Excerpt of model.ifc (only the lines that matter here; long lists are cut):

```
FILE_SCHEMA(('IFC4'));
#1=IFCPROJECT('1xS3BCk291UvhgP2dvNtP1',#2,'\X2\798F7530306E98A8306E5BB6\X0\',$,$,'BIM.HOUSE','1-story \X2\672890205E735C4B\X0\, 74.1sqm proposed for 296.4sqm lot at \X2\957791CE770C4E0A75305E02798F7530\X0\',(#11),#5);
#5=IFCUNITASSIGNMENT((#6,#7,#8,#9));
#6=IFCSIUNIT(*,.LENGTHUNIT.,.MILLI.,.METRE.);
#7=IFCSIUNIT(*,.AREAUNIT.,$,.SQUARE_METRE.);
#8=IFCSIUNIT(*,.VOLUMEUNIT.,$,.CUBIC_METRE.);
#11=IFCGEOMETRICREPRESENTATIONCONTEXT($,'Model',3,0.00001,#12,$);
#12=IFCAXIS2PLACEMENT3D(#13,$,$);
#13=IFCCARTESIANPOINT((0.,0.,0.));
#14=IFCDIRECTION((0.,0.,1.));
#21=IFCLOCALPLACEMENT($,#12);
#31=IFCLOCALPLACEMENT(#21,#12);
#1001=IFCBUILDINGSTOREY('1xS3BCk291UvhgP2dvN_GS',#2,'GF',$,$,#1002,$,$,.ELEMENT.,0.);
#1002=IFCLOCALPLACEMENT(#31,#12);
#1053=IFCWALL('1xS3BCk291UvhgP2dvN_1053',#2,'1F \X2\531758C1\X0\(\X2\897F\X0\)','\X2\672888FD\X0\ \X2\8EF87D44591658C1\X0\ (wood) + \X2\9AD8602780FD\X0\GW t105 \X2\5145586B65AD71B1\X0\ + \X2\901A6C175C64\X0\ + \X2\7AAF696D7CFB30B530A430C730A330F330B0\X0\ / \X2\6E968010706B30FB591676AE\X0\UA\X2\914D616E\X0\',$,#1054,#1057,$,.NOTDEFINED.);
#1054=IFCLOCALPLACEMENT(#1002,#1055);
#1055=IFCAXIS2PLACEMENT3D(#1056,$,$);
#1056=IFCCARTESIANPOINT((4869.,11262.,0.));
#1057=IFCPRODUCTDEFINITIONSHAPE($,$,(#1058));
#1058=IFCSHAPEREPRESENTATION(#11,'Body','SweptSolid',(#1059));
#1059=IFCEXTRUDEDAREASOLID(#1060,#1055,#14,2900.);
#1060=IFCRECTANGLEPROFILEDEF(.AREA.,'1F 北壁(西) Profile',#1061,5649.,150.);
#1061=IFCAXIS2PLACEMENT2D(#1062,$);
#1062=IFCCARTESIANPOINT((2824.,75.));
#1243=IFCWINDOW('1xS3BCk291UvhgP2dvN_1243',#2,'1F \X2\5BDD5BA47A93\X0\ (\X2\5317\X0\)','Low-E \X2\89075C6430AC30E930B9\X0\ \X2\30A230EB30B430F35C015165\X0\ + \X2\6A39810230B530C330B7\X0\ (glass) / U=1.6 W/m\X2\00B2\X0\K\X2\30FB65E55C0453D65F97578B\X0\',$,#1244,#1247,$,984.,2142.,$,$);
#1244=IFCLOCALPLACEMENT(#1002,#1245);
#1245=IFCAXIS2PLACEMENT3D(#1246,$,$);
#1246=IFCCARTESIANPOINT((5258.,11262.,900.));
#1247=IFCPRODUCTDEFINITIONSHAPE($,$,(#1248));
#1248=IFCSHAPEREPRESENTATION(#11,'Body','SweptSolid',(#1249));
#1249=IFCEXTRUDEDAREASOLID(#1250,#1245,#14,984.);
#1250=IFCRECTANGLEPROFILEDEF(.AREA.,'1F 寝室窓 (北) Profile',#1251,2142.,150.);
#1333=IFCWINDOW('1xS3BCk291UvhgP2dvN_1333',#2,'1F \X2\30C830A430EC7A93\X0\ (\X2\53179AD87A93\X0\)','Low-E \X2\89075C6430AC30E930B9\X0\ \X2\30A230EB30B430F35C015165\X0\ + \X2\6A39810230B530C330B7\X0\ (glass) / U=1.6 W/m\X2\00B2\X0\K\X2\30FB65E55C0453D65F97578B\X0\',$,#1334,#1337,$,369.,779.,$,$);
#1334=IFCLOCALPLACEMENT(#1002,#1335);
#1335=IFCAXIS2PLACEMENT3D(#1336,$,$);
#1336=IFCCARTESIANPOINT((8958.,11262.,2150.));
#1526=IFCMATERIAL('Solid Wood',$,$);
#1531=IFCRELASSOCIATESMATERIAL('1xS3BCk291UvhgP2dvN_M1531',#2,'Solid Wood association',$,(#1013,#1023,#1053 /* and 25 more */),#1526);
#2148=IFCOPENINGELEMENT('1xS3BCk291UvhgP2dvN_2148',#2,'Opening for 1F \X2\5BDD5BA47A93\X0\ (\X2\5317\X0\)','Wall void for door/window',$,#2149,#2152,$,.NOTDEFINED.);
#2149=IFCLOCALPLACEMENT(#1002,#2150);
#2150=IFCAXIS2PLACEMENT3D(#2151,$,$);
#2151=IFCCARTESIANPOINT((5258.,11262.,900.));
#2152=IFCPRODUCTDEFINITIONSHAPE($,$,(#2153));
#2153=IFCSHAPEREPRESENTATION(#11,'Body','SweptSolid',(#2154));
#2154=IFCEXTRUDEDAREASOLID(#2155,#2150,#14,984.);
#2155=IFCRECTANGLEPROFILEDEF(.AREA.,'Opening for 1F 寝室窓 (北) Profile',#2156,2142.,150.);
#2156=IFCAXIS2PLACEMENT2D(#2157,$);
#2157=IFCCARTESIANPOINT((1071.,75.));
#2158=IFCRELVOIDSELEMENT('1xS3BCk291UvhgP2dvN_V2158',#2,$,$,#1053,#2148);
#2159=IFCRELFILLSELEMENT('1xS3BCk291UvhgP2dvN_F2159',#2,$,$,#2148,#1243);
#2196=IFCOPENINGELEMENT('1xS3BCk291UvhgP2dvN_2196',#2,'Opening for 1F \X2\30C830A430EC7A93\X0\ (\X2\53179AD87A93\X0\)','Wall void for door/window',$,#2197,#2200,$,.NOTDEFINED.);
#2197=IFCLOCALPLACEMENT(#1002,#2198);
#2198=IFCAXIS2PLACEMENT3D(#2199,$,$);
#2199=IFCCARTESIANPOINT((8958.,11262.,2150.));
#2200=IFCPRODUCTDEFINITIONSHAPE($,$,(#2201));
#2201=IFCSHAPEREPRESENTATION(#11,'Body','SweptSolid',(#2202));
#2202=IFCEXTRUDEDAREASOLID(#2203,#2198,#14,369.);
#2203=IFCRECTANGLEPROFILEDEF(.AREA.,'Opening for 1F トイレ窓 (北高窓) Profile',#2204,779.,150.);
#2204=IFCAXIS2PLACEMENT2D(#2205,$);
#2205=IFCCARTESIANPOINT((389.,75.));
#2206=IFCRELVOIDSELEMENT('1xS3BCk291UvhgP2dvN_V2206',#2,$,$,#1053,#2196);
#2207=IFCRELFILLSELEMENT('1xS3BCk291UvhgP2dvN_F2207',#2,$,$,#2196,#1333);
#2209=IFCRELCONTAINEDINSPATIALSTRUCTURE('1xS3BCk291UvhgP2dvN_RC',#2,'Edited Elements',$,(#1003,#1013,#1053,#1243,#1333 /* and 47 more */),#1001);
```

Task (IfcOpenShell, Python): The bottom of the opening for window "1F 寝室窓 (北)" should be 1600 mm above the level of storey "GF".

```python
import numpy as np
import ifcopenshell
import ifcopenshell.api.geometry
import ifcopenshell.geom
import ifcopenshell.util.element
import ifcopenshell.util.placement
import ifcopenshell.util.shape
import ifcopenshell.util.unit

model = ifcopenshell.open("model.ifc")
unit_scale = ifcopenshell.util.unit.calculate_unit_scale(model)

window = model.by_guid("1xS3BCk291UvhgP2dvN_1243")
opening = window.FillsVoids[0].RelatingOpeningElement
storey = ifcopenshell.util.element.get_container(window, ifc_class="IfcBuildingStorey")
level = ifcopenshell.util.placement.get_local_placement(storey.ObjectPlacement)[2, 3]

# The opening's origin need not be at the sill, so measure its lowest point.
shape = ifcopenshell.geom.create_shape(ifcopenshell.geom.settings(), opening)
bottom = ifcopenshell.util.shape.get_shape_bottom_elevation(shape, shape.geometry) / unit_scale
dz = level + 1.6 / unit_scale - bottom

shift = np.array([0.0, 0.0, dz])
# The window is not placed relative to its opening, so move both.
for product in (opening, window):
    matrix = ifcopenshell.util.placement.get_local_placement(product.ObjectPlacement)
    matrix[:3, 3] += shift
    ifcopenshell.api.geometry.edit_object_placement(model, product=product, matrix=matrix, is_si=False)

print(f"moved by {dz * unit_scale:+.3f} m")

model.write("model_rev.ifc")
```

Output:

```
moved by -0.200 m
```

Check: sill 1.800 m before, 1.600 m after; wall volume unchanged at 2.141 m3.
